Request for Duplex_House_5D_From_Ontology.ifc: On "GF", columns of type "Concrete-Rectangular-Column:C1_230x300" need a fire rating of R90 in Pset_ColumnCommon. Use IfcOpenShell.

First a look at what the model holds.

```python
import ifcopenshell
import ifcopenshell.util.element

model = ifcopenshell.open("Duplex_House_5D_From_Ontology.ifc")
print(model.schema)
storey = next(s for s in model.by_type("IfcBuildingStorey") if s.Name == "GF")
columns = [e for e in ifcopenshell.util.element.get_decomposition(storey) if e.is_a("IfcColumn")]
seen = {}
for e in columns:
    element_type = ifcopenshell.util.element.get_type(e)
    key = (element_type.Name if element_type != e and element_type else None, ifcopenshell.util.element.get_pset(e, "Pset_ColumnCommon", "FireRating"))
    seen[key] = seen.get(key, 0) + 1
for (name, value), count in sorted(seen.items(), key=str):
    print(count, "x", name, "|", value)
```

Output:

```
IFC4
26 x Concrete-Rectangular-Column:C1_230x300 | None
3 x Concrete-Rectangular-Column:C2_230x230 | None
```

```python
import ifcopenshell
import ifcopenshell.api.pset
import ifcopenshell.util.element

model = ifcopenshell.open("Duplex_House_5D_From_Ontology.ifc")

storey = next(s for s in model.by_type("IfcBuildingStorey") if s.Name == "GF")
columns = [e for e in ifcopenshell.util.element.get_decomposition(storey) if e.is_a("IfcColumn")]

count = 0
for e in columns:
    element_type = ifcopenshell.util.element.get_type(e)
    if element_type in (None, e) or element_type.Name != "Concrete-Rectangular-Column:C1_230x300":
        continue
    # add_pset returns the element's existing set when there is one.
    pset = ifcopenshell.api.pset.add_pset(model, product=e, name="Pset_ColumnCommon")
    ifcopenshell.api.pset.edit_pset(model, pset=pset, properties={"FireRating": "R90"})
    count += 1

print(count, "columns updated")

model.write("Duplex_House_5D_From_Ontology_rev.ifc")
```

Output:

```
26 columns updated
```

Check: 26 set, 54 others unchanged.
